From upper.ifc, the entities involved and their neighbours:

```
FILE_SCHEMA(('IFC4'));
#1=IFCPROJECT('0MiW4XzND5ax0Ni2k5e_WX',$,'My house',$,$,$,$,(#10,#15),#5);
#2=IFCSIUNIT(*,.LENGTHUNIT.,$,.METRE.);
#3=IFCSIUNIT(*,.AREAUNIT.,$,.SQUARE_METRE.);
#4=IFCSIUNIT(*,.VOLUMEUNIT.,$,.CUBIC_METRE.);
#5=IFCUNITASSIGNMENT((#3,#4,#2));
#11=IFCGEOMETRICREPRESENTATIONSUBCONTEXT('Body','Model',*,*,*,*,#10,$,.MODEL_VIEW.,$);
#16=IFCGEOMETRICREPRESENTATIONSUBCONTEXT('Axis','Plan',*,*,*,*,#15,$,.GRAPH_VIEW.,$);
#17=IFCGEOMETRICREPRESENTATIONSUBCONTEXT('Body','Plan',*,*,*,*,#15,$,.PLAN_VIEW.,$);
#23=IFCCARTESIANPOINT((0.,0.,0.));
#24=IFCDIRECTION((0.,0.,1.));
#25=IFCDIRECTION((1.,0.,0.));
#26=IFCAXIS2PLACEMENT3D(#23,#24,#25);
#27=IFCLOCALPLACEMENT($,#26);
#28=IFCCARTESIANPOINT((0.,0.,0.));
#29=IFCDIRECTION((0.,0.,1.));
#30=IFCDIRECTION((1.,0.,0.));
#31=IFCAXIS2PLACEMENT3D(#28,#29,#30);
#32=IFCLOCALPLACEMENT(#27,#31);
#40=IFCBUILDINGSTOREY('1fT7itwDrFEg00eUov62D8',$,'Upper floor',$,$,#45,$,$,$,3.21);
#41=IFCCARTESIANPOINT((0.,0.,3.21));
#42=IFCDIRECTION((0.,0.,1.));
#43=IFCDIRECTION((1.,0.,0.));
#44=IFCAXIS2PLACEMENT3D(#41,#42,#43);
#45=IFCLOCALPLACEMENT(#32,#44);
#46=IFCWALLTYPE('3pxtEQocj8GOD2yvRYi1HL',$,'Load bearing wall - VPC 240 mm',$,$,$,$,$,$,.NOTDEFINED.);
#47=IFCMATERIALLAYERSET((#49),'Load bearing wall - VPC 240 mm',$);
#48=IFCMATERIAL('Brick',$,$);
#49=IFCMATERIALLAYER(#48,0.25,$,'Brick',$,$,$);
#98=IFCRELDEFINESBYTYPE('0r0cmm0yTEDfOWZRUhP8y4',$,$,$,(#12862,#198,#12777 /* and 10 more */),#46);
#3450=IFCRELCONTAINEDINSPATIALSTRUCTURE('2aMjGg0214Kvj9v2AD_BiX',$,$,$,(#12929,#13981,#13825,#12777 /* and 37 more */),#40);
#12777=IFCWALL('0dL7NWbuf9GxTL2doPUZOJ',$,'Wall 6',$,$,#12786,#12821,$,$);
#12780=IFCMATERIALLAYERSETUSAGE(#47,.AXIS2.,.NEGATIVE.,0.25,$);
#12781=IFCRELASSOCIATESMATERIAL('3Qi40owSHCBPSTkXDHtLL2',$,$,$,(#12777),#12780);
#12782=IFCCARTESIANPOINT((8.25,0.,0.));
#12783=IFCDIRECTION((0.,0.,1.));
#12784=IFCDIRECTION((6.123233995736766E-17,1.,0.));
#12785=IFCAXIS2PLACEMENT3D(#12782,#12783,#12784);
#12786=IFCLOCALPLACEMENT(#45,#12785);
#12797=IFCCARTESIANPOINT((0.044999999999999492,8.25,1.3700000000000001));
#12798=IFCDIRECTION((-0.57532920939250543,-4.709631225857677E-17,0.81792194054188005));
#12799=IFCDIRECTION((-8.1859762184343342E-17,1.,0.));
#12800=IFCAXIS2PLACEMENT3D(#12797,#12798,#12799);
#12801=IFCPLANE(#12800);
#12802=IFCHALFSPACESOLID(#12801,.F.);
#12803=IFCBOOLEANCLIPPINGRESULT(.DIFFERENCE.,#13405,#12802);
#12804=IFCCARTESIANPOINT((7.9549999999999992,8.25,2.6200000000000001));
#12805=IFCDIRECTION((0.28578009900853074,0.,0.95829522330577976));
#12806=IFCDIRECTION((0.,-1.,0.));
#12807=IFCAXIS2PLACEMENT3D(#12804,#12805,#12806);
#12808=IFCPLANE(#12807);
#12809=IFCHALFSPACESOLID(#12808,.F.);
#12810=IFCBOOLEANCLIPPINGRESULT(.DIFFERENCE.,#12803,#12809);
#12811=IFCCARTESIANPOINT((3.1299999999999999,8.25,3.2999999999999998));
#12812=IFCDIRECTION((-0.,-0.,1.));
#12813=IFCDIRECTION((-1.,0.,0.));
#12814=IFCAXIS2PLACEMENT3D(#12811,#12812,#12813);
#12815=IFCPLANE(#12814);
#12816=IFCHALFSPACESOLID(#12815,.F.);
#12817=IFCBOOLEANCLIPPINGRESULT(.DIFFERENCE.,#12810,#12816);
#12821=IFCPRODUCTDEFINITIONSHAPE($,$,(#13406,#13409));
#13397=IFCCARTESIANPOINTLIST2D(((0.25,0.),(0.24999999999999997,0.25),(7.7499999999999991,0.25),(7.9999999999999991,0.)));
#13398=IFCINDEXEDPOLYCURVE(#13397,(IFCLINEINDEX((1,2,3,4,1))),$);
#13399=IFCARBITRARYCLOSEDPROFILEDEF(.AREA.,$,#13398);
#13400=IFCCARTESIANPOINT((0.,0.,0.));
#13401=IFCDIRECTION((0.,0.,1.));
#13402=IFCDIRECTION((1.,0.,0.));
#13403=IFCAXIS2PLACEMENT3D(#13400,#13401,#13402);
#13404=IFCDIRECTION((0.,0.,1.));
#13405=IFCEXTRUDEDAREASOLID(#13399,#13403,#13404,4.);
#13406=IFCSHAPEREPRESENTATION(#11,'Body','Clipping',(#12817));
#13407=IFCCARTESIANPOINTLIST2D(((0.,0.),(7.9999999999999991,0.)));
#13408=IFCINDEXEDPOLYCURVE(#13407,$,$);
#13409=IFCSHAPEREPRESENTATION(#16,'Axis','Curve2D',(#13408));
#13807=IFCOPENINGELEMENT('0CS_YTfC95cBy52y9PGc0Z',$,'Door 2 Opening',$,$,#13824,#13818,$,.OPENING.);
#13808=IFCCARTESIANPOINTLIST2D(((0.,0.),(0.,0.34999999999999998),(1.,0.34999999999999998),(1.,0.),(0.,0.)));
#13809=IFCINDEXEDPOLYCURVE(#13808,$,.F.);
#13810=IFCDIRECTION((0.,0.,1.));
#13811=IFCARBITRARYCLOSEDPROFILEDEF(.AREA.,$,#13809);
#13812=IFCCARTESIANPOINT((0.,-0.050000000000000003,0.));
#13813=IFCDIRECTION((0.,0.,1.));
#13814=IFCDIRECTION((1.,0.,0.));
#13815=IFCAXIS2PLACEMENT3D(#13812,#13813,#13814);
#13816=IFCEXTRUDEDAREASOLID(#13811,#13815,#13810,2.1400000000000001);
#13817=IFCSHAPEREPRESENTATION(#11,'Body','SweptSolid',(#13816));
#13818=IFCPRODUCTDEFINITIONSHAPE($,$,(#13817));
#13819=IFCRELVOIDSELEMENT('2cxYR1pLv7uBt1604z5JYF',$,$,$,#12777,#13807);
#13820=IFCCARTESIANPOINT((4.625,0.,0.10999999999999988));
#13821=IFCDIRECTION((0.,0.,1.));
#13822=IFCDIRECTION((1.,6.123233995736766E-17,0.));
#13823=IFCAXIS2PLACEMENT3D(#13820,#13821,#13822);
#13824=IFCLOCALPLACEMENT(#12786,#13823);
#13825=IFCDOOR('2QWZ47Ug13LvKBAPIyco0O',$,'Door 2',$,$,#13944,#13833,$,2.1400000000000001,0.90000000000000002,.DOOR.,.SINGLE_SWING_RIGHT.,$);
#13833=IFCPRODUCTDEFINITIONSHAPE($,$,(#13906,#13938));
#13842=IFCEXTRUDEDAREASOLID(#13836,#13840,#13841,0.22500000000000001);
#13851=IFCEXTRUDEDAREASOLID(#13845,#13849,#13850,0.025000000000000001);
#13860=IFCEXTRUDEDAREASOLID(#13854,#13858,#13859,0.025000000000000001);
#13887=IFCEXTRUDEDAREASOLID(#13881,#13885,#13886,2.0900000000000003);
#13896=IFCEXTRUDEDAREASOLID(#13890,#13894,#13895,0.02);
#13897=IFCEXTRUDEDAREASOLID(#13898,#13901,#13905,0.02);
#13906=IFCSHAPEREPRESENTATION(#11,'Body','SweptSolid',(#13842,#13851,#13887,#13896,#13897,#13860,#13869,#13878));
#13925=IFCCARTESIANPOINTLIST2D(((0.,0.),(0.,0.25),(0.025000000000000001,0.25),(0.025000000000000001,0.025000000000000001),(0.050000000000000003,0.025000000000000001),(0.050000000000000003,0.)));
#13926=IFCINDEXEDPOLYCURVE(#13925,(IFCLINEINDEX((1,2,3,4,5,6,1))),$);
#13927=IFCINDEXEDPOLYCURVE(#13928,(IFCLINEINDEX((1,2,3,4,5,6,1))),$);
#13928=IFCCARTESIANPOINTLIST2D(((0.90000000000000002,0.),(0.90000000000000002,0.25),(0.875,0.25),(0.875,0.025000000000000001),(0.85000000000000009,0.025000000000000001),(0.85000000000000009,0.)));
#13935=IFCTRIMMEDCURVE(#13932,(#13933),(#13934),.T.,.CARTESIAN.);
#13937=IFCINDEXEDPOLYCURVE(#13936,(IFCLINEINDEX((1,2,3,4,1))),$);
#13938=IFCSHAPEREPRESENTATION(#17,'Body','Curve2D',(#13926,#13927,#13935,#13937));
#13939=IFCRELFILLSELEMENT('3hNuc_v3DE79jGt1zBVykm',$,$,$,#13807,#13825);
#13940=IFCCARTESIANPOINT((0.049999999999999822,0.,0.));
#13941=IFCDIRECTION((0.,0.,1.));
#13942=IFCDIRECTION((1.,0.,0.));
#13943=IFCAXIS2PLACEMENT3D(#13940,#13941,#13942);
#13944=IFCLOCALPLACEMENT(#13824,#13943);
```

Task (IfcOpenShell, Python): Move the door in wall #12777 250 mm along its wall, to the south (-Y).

```python
import ifcopenshell
import ifcopenshell.api.geometry
import ifcopenshell.util.placement
import ifcopenshell.util.unit

model = ifcopenshell.open("upper.ifc")
unit_scale = ifcopenshell.util.unit.calculate_unit_scale(model)

door = model.by_guid("2QWZ47Ug13LvKBAPIyco0O")
opening = door.FillsVoids[0].RelatingOpeningElement
wall = opening.VoidsElements[0].RelatingBuildingElement

wall_matrix = ifcopenshell.util.placement.get_local_placement(wall.ObjectPlacement)
shift = wall_matrix[:3, 0] * -0.25 / unit_scale
before = ifcopenshell.util.placement.get_local_placement(door.ObjectPlacement)[:3, 3].copy()

# The door is placed relative to its opening, so it follows when the opening moves.
matrix = ifcopenshell.util.placement.get_local_placement(opening.ObjectPlacement)
matrix[:3, 3] += shift
ifcopenshell.api.geometry.edit_object_placement(
    model, product=opening, matrix=matrix, is_si=False, should_transform_children=True
)

after = ifcopenshell.util.placement.get_local_placement(door.ObjectPlacement)[:3, 3]
print("door moved by", (after - before).round(3) + 0.0)

model.write("upper_v2.ifc")
```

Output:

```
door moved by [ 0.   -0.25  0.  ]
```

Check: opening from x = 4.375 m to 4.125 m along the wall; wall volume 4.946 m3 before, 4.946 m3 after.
